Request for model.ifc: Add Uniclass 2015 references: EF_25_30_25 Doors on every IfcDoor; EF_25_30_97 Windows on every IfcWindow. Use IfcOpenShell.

First a look at what the model holds.

```python
import ifcopenshell

model = ifcopenshell.open("model.ifc")
print(model.schema)
print("classifications:", [c.Name for c in model.by_type("IfcClassification")])
for ifc_class in ("IfcDoor", "IfcRoof", "IfcStair", "IfcWall", "IfcWindow"):
    print(ifc_class, len(model.by_type(ifc_class)))
```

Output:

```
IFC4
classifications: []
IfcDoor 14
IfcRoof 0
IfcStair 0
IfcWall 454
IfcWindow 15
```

```python
import ifcopenshell
import ifcopenshell.api.classification

model = ifcopenshell.open("model.ifc")

system = ifcopenshell.api.classification.add_classification(model, classification="Uniclass 2015")

codes = {
    "IfcDoor": ("EF_25_30_25", "Doors"),
    "IfcWindow": ("EF_25_30_97", "Windows"),
}
for ifc_class, (code, name) in codes.items():
    products = model.by_type(ifc_class)
    ifcopenshell.api.classification.add_reference(
        model, products=products, classification=system, identification=code, name=name
    )
    print(code, len(products))

model.write("model_updated.ifc")
```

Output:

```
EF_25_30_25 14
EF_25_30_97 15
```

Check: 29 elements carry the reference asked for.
